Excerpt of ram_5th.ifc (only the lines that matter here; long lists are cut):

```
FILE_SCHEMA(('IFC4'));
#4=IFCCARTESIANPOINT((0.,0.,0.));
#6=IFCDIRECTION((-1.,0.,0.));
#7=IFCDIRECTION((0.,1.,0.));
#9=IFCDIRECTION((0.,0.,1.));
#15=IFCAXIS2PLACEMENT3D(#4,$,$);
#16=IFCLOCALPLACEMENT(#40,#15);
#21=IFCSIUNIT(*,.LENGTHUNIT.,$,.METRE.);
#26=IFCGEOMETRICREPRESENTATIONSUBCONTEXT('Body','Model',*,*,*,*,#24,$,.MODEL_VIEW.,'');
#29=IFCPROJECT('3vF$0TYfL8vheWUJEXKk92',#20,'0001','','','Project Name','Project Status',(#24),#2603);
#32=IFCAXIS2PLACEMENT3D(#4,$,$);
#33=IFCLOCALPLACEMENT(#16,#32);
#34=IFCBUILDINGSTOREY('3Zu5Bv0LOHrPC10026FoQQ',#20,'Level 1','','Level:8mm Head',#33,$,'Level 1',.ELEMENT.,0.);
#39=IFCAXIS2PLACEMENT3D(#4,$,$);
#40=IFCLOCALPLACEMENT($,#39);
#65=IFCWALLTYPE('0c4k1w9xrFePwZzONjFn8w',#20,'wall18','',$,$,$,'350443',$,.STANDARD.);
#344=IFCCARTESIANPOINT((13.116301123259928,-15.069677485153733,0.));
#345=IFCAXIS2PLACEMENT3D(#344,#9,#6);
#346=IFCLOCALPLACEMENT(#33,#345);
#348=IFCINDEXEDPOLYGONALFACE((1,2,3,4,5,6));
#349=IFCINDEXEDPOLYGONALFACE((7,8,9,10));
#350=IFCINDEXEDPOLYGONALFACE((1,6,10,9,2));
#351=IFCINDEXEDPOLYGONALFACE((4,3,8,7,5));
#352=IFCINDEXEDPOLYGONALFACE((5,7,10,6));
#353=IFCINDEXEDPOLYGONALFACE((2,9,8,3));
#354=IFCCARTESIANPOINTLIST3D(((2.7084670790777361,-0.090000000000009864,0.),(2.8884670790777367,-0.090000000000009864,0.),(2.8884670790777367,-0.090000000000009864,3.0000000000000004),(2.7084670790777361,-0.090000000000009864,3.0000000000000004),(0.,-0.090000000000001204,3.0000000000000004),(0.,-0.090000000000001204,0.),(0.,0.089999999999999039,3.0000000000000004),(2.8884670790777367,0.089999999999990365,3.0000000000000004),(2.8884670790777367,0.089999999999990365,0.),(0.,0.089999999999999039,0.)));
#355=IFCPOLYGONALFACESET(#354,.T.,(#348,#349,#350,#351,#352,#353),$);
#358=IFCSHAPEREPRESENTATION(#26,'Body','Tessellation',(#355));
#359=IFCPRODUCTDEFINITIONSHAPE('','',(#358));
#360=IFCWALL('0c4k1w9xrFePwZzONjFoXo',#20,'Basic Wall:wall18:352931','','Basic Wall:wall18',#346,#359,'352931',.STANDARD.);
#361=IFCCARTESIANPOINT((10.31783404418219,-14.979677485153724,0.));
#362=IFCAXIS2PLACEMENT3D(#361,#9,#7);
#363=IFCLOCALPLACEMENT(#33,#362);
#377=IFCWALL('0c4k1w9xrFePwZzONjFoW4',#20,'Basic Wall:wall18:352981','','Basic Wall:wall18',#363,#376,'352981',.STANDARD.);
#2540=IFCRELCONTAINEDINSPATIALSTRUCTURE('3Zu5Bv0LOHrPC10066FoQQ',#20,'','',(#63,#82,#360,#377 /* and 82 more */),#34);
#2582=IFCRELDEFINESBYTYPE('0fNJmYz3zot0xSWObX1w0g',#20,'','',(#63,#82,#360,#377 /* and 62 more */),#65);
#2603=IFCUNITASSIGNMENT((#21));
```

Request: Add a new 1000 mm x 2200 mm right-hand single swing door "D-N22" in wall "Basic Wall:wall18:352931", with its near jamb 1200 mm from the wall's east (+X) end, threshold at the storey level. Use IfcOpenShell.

```python
import numpy as np
import ifcopenshell
import ifcopenshell.api.feature
import ifcopenshell.api.geometry
import ifcopenshell.api.root
import ifcopenshell.api.spatial
import ifcopenshell.geom
import ifcopenshell.util.element
import ifcopenshell.util.placement
import ifcopenshell.util.representation
import ifcopenshell.util.shape
import ifcopenshell.util.unit

model = ifcopenshell.open("ram_5th.ifc")
unit_scale = ifcopenshell.util.unit.calculate_unit_scale(model)
settings = ifcopenshell.geom.settings()


def volume(element):
    """Net volume in cubic metres, openings subtracted."""
    shape = ifcopenshell.geom.create_shape(settings, element)
    return ifcopenshell.util.shape.get_volume(shape.geometry)


wall = model.by_guid("0c4k1w9xrFePwZzONjFoXo")
storey = ifcopenshell.util.element.get_container(wall, ifc_class="IfcBuildingStorey")
context = ifcopenshell.util.representation.get_context(model, "Model", "Body", "MODEL_VIEW")
before = volume(wall)

width, height, from_end, sill = 1, 2.2, 1.2, 0.0  # metres

# The wall runs along its own X axis, and the end named is its -X end.
wall_shape = ifcopenshell.geom.create_shape(settings, wall)
x, y, z = ifcopenshell.util.shape.get_vertices(wall_shape.geometry).T
start = x.min() + from_end
face, thickness = float(y.min()), float(y.max() - y.min())
wall_matrix = ifcopenshell.util.placement.get_local_placement(wall.ObjectPlacement)
level = ifcopenshell.util.placement.get_local_placement(storey.ObjectPlacement)[2, 3]


def in_wall(x, y):
    """Placement at x, y metres in the wall's axes, at sill height."""
    matrix = wall_matrix.copy()
    matrix[:, 3] = wall_matrix @ np.array([x / unit_scale, y / unit_scale, 0.0, 1.0])
    matrix[2, 3] = level + sill / unit_scale
    return matrix


# Opening: a box that overshoots both wall faces by 50 mm.
opening = ifcopenshell.api.root.create_entity(model, ifc_class="IfcOpeningElement", predefined_type="OPENING")
box = ifcopenshell.api.geometry.add_wall_representation(
    model, context=context, length=width, height=height, thickness=thickness + 0.1
)
ifcopenshell.api.geometry.assign_representation(model, product=opening, representation=box)
ifcopenshell.api.geometry.edit_object_placement(model, product=opening, matrix=in_wall(start, face - 0.05), is_si=False)
ifcopenshell.api.feature.add_feature(model, feature=opening, element=wall)

door = ifcopenshell.api.root.create_entity(model, ifc_class="IfcDoor", name="D-N22", predefined_type="DOOR")
door.OverallWidth, door.OverallHeight = width / unit_scale, height / unit_scale
door.OperationType = "SINGLE_SWING_RIGHT"
body = ifcopenshell.api.geometry.add_door_representation(
    model,
    context=context,
    overall_width=door.OverallWidth,
    overall_height=door.OverallHeight,
    operation_type="SINGLE_SWING_RIGHT",
    lining_properties={"LiningDepth": thickness / unit_scale, "ThresholdDepth": thickness / unit_scale},
)
ifcopenshell.api.geometry.assign_representation(model, product=door, representation=body)
ifcopenshell.api.spatial.assign_container(model, products=[door], relating_structure=storey)
ifcopenshell.api.feature.add_filling(model, opening=opening, element=door)

# The lining spans the wall, so the door starts at the wall face.
ifcopenshell.api.geometry.edit_object_placement(model, product=door, matrix=in_wall(start, face), is_si=False)

after = volume(wall)

print(f"wall volume {before:.3f} -> {after:.3f} m3")

model.write("ram_5th_rev.ifc")
```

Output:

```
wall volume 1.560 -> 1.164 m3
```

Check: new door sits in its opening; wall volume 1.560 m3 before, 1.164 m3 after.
